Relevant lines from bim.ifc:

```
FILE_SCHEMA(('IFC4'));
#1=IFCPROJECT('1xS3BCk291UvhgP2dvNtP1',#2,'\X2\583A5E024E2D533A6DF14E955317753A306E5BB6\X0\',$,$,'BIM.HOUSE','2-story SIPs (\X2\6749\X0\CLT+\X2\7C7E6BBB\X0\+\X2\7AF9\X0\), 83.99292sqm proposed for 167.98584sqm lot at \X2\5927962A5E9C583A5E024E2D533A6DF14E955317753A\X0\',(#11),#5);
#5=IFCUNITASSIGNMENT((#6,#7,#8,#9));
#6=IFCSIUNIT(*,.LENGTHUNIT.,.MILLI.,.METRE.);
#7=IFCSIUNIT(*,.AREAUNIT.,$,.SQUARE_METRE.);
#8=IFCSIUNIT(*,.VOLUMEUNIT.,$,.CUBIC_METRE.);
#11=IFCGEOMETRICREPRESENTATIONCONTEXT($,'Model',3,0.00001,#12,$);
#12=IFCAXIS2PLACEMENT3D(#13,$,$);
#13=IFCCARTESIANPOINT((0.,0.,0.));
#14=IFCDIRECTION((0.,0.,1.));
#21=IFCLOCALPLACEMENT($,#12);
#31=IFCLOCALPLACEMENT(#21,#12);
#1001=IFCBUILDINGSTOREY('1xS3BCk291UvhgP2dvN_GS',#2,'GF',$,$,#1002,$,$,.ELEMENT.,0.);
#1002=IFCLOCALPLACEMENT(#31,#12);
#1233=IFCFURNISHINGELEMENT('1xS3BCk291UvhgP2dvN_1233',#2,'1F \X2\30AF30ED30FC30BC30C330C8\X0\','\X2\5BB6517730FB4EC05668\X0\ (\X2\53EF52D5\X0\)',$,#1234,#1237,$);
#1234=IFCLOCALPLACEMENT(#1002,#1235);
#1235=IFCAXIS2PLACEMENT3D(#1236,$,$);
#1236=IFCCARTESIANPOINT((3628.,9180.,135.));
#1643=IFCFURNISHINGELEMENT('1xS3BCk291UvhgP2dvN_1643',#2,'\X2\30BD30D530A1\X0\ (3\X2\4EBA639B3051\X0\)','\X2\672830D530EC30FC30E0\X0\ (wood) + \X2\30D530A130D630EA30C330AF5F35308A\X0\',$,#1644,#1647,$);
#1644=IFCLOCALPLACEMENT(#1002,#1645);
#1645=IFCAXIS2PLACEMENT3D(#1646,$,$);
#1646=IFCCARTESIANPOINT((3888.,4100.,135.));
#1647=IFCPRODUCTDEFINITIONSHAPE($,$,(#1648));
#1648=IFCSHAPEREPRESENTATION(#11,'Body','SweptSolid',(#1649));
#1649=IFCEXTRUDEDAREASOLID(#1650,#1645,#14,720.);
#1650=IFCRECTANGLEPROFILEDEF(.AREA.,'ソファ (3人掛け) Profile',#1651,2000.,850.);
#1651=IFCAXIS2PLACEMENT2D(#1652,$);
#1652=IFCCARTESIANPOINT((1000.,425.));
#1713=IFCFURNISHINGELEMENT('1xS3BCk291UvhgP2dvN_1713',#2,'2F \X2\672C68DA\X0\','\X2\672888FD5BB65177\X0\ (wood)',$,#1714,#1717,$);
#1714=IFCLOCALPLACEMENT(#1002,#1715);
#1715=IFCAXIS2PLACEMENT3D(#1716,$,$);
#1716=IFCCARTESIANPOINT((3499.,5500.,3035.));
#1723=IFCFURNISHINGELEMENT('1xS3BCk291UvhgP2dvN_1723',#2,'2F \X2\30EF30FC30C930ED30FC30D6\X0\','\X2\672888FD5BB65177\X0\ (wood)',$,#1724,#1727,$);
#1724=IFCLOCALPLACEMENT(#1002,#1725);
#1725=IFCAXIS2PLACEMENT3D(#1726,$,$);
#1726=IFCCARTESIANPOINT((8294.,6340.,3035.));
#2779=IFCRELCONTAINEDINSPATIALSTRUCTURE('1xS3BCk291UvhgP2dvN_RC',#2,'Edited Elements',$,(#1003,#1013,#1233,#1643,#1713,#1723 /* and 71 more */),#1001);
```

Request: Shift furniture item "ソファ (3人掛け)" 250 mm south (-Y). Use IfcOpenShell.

```python
import ifcopenshell
import ifcopenshell.api.geometry
import ifcopenshell.util.placement

model = ifcopenshell.open("bim.ifc")

item = model.by_guid("1xS3BCk291UvhgP2dvN_1643")
matrix = ifcopenshell.util.placement.get_local_placement(item.ObjectPlacement)
matrix[1, 3] -= 250.0
ifcopenshell.api.geometry.edit_object_placement(model, product=item, matrix=matrix, is_si=False)

print(ifcopenshell.util.placement.get_local_placement(item.ObjectPlacement).round(3) + 0.0)

model.write("bim_edited.ifc")
```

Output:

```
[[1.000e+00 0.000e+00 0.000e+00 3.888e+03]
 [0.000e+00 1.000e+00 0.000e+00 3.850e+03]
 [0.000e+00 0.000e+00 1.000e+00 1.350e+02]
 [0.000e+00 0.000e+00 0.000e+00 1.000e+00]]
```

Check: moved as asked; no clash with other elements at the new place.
